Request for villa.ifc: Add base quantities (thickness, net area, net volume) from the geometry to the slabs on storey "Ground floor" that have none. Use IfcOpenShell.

First a look at what the model holds.

```python
import ifcopenshell
import ifcopenshell.util.element
import ifcopenshell.util.unit

model = ifcopenshell.open("villa.ifc")
print(model.schema)
for unit_type in ("LENGTHUNIT", "AREAUNIT", "VOLUMEUNIT"):
    print(unit_type, ifcopenshell.util.unit.calculate_unit_scale(model, unit_type))
storey = next(s for s in model.by_type("IfcBuildingStorey") if s.Name == "Ground floor")
slabs = [e for e in ifcopenshell.util.element.get_decomposition(storey) if e.is_a("IfcSlab")]
for e in sorted(slabs, key=lambda e: e.id()):
    print(e.id(), e.is_a(), e.Name, list(ifcopenshell.util.element.get_psets(e, qtos_only=True)), sep=" | ")
```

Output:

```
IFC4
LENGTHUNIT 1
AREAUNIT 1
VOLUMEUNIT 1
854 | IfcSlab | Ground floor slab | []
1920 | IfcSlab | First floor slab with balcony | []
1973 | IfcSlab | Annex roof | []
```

```python
import ifcopenshell
import ifcopenshell.api.pset
import ifcopenshell.geom
import ifcopenshell.util.element
import ifcopenshell.util.shape
import ifcopenshell.util.unit

model = ifcopenshell.open("villa.ifc")
unit_scale = ifcopenshell.util.unit.calculate_unit_scale(model)
area_scale = ifcopenshell.util.unit.calculate_unit_scale(model, "AREAUNIT")
volume_scale = ifcopenshell.util.unit.calculate_unit_scale(model, "VOLUMEUNIT")
settings = ifcopenshell.geom.settings()

storey = next(s for s in model.by_type("IfcBuildingStorey") if s.Name == "Ground floor")
slabs = [e for e in ifcopenshell.util.element.get_decomposition(storey) if e.is_a("IfcSlab")]

for e in sorted(slabs, key=lambda e: e.id()):
    if ifcopenshell.util.element.get_psets(e, qtos_only=True, should_inherit=False):
        continue
    # Geometry comes back in metres, in the element's own axes.
    shape = ifcopenshell.geom.create_shape(settings, e)
    values = {
        "Width": ifcopenshell.util.shape.get_z(shape.geometry) / unit_scale,
        "NetArea": ifcopenshell.util.shape.get_footprint_area(shape.geometry) / area_scale,
        "NetVolume": ifcopenshell.util.shape.get_volume(shape.geometry) / volume_scale,
    }
    qto = ifcopenshell.api.pset.add_qto(model, product=e, name="Qto_SlabBaseQuantities")
    ifcopenshell.api.pset.edit_qto(model, qto=qto, properties=values)
    print(e.id(), {k: round(v, 3) for k, v in values.items()})

model.write("villa_v2.ifc")
```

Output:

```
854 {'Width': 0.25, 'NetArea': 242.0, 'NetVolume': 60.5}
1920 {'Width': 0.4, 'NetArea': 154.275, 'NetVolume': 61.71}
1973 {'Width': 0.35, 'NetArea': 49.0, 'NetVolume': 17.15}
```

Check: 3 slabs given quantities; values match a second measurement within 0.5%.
